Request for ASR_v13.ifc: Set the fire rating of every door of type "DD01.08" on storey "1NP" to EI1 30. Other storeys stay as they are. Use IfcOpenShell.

First a look at what the model holds.

```python
import ifcopenshell
import ifcopenshell.util.element

model = ifcopenshell.open("ASR_v13.ifc")
print(model.schema)
storey = next(s for s in model.by_type("IfcBuildingStorey") if s.Name == "1NP")
doors = [e for e in ifcopenshell.util.element.get_decomposition(storey) if e.is_a("IfcDoor")]
seen = {}
for e in doors:
    element_type = ifcopenshell.util.element.get_type(e)
    key = (element_type.Name if element_type != e and element_type else None, ifcopenshell.util.element.get_pset(e, "Pset_DoorCommon", "FireRating"))
    seen[key] = seen.get(key, 0) + 1
for (name, value), count in sorted(seen.items(), key=str):
    print(count, "x", name, "|", value)
```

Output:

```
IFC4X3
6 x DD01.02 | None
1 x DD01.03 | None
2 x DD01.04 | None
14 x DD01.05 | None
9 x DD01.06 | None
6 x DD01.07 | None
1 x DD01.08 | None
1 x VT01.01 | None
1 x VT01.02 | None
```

```python
import ifcopenshell
import ifcopenshell.api.pset
import ifcopenshell.util.element

model = ifcopenshell.open("ASR_v13.ifc")

storey = next(s for s in model.by_type("IfcBuildingStorey") if s.Name == "1NP")
doors = [e for e in ifcopenshell.util.element.get_decomposition(storey) if e.is_a("IfcDoor")]

count = 0
for e in doors:
    element_type = ifcopenshell.util.element.get_type(e)
    if element_type in (None, e) or element_type.Name != "DD01.08":
        continue
    # add_pset returns the element's existing set when there is one.
    pset = ifcopenshell.api.pset.add_pset(model, product=e, name="Pset_DoorCommon")
    ifcopenshell.api.pset.edit_pset(model, pset=pset, properties={"FireRating": "EI1 30"})
    count += 1

print(count, "doors updated")

model.write("ASR_v13_v2.ifc")
```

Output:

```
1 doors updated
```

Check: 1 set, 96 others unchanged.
